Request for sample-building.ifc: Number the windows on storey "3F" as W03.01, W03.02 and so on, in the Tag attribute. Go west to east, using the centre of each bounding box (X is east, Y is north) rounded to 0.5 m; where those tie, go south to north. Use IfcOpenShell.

First a look at what the model holds.

```python
import ifcopenshell
import ifcopenshell.util.element
import ifcopenshell.util.placement

model = ifcopenshell.open("sample-building.ifc")
print(model.schema)
storey = next(s for s in model.by_type("IfcBuildingStorey") if s.Name == "3F")
windows = [e for e in ifcopenshell.util.element.get_decomposition(storey) if e.is_a("IfcWindow")]
for e in sorted(windows, key=lambda e: e.id()):
    origin = ifcopenshell.util.placement.get_local_placement(e.ObjectPlacement)[:3, 3]
    print(e.id(), e.Tag, e.Name, origin.round(2) + 0.0, sep=" | ")
```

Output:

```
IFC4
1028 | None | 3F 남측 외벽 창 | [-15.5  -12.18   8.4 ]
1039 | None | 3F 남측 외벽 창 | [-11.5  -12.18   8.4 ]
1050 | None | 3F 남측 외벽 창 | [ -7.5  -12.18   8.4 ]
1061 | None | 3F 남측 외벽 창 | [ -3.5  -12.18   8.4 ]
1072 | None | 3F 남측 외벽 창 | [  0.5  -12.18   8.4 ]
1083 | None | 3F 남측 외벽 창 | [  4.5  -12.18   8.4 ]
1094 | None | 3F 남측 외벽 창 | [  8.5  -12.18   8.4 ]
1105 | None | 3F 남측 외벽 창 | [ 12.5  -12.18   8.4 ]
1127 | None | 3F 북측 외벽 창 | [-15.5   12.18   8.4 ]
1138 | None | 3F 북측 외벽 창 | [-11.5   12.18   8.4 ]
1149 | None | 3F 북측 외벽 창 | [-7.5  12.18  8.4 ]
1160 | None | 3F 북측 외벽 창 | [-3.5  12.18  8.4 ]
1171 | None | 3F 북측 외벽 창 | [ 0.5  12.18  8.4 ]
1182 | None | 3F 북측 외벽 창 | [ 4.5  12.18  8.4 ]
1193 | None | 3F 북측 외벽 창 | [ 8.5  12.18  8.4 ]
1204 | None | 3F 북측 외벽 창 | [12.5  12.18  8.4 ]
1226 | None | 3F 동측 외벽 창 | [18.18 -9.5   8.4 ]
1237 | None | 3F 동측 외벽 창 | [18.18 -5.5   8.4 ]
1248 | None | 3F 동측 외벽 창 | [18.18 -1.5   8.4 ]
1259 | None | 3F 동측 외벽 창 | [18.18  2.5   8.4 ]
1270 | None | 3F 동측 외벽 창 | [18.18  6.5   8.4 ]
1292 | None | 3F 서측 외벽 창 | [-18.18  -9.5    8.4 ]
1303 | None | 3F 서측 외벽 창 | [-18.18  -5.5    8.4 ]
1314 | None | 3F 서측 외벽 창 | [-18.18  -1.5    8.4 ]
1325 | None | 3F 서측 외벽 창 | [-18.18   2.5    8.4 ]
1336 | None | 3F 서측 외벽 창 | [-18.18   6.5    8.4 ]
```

```python
import ifcopenshell
import ifcopenshell.geom
import ifcopenshell.util.element
import ifcopenshell.util.shape

model = ifcopenshell.open("sample-building.ifc")
settings = ifcopenshell.geom.settings()
settings.set("use-world-coords", True)


def centre(element):
    shape = ifcopenshell.geom.create_shape(settings, element)
    return ifcopenshell.util.shape.get_bbox_centroid(shape.geometry)


storey = next(s for s in model.by_type("IfcBuildingStorey") if s.Name == "3F")
windows = [e for e in ifcopenshell.util.element.get_decomposition(storey) if e.is_a("IfcWindow")]

# Insertion points can sit at a corner or the storey origin, so sort by the geometry (in metres).
centres = {e: centre(e) for e in windows}
windows.sort(key=lambda e: (round(centres[e][0] / 0.5), centres[e][1]))

for i, e in enumerate(windows, start=1):
    number = f"W03.{i:02d}"
    e.Tag = number
    print(e.id(), number)

model.write("sample-building_v2.ifc")
```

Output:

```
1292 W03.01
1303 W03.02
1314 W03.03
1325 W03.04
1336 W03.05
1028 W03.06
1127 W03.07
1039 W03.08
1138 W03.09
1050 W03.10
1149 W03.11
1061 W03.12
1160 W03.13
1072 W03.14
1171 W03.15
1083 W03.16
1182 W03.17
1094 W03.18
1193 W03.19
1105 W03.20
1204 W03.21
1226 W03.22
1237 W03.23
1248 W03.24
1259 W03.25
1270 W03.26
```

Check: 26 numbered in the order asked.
